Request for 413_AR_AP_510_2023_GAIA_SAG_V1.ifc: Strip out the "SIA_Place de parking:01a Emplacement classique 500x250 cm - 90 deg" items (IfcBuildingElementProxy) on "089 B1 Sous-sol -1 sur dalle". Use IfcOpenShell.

First a look at what the model holds.

```python
import ifcopenshell
import ifcopenshell.util.element

model = ifcopenshell.open("413_AR_AP_510_2023_GAIA_SAG_V1.ifc")
print(model.schema)
storey = next(s for s in model.by_type("IfcBuildingStorey") if s.Name == "089 B1 Sous-sol -1 sur dalle")
proxies = [e for e in ifcopenshell.util.element.get_decomposition(storey) if e.is_a("IfcBuildingElementProxy")]
seen = {}
for e in proxies:
    element_type = ifcopenshell.util.element.get_type(e)
    name = element_type.Name if element_type not in (None, e) else None
    seen[name] = seen.get(name, 0) + 1
for name, count in sorted(seen.items(), key=str):
    print(count, "x", name)
```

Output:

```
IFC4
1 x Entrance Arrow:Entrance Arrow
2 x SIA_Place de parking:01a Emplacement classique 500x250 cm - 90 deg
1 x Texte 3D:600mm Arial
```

```python
import ifcopenshell
import ifcopenshell.api.root
import ifcopenshell.util.element

model = ifcopenshell.open("413_AR_AP_510_2023_GAIA_SAG_V1.ifc")

storey = next(s for s in model.by_type("IfcBuildingStorey") if s.Name == "089 B1 Sous-sol -1 sur dalle")
proxies = [e for e in ifcopenshell.util.element.get_decomposition(storey) if e.is_a("IfcBuildingElementProxy")]
targets = [e for e in proxies if (t := ifcopenshell.util.element.get_type(e)) not in (None, e) and t.Name == "SIA_Place de parking:01a Emplacement classique 500x250 cm - 90 deg"]

for e in targets:
    ifcopenshell.api.root.remove_product(model, product=e)
print(len(targets), "removed")

model.write("413_AR_AP_510_2023_GAIA_SAG_V1_edited.ifc")
```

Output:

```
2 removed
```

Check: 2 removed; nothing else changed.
